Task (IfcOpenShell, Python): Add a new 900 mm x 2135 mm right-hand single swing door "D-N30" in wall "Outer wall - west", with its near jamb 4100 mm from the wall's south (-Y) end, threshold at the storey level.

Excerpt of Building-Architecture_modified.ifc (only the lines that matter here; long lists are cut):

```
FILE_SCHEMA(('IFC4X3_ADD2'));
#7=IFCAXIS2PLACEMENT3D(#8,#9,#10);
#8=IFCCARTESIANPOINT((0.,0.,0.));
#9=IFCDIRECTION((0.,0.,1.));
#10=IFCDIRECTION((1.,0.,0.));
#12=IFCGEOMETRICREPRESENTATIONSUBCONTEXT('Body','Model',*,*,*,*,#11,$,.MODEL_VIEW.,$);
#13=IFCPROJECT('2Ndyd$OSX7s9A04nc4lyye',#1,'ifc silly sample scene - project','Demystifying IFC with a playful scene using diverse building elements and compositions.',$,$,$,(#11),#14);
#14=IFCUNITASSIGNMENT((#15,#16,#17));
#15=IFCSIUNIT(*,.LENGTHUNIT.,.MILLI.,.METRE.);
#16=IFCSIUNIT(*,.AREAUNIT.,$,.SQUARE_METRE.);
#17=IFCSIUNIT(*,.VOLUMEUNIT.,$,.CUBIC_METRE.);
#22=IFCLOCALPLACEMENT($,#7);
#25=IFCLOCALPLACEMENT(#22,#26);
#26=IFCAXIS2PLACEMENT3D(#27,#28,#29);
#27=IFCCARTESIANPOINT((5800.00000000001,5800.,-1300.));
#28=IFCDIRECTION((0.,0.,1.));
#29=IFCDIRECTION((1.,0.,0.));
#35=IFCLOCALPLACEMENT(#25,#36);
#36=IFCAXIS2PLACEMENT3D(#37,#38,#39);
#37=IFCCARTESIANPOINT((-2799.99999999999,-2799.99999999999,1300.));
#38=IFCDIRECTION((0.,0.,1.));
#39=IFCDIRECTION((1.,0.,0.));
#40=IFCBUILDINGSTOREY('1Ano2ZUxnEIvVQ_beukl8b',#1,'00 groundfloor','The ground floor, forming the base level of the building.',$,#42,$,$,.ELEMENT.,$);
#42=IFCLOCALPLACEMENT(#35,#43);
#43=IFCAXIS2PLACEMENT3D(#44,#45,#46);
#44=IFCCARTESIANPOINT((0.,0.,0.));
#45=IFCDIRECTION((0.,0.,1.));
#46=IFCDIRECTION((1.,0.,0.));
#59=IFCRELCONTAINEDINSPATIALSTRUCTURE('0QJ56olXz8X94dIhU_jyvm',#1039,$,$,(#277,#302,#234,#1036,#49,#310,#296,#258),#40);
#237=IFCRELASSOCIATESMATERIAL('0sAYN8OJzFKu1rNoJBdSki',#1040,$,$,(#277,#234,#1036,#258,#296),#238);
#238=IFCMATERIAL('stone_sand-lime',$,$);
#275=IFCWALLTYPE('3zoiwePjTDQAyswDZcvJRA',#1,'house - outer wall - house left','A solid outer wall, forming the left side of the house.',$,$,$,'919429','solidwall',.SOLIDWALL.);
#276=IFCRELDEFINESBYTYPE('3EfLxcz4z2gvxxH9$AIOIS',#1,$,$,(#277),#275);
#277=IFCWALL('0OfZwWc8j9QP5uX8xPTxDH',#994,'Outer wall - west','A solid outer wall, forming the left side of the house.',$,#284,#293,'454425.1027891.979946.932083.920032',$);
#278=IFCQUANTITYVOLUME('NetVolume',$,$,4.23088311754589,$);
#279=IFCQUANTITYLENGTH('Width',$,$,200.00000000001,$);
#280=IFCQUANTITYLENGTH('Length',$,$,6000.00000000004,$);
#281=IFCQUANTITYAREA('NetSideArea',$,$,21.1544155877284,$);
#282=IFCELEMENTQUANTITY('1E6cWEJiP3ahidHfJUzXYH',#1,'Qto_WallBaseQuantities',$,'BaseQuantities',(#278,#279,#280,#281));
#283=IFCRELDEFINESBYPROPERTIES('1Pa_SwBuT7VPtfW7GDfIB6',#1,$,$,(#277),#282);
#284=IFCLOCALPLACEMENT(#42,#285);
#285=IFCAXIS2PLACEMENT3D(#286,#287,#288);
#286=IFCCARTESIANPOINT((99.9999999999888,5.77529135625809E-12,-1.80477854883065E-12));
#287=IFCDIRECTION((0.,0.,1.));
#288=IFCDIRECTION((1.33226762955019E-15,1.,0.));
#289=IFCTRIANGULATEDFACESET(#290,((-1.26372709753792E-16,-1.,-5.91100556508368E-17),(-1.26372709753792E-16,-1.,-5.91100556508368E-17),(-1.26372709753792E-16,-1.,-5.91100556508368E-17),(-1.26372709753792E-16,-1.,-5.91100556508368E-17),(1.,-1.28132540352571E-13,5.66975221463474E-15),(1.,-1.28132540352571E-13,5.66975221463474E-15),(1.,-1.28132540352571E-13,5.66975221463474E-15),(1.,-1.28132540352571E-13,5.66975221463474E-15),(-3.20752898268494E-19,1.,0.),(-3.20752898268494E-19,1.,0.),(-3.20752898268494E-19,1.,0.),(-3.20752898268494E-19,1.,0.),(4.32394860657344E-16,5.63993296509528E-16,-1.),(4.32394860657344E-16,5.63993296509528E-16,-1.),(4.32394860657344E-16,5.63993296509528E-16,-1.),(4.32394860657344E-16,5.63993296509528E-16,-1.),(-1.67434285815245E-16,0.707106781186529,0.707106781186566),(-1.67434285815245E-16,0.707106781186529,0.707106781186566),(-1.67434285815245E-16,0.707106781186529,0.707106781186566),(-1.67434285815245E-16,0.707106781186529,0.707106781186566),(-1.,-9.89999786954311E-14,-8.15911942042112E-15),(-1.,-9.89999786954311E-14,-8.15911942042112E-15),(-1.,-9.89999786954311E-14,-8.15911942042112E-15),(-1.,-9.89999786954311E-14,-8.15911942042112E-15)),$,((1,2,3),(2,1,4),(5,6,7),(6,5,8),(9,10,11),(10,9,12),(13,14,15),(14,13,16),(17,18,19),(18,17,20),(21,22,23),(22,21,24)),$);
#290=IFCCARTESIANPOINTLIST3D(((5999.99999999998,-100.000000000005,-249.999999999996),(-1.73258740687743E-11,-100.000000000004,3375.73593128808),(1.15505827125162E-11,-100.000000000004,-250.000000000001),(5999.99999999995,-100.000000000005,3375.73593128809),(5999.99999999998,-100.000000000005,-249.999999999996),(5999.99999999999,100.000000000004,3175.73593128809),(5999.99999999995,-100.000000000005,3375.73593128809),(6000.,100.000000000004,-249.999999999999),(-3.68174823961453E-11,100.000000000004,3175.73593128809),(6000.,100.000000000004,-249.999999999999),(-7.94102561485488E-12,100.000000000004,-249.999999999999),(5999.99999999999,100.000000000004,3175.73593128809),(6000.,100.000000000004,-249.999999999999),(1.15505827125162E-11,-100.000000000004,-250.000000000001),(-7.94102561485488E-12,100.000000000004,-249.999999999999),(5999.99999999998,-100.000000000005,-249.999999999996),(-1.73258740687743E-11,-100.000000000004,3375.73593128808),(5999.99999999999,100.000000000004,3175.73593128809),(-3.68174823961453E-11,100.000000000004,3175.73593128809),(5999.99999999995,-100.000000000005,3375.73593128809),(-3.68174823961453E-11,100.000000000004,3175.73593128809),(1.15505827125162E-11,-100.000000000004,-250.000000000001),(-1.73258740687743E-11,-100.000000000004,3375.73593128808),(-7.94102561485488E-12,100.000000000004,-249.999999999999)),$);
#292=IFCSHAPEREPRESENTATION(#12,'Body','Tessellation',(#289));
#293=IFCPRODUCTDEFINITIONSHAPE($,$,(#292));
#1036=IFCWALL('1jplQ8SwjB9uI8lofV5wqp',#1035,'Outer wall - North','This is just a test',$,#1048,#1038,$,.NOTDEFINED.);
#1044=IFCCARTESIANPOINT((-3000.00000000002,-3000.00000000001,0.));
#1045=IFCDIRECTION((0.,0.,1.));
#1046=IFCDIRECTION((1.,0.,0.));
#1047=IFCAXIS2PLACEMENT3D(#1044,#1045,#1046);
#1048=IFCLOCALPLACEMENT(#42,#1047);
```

```python
import numpy as np
import ifcopenshell
import ifcopenshell.api.feature
import ifcopenshell.api.geometry
import ifcopenshell.api.pset
import ifcopenshell.api.root
import ifcopenshell.api.spatial
import ifcopenshell.geom
import ifcopenshell.util.element
import ifcopenshell.util.placement
import ifcopenshell.util.representation
import ifcopenshell.util.shape
import ifcopenshell.util.unit

model = ifcopenshell.open("Building-Architecture_modified.ifc")
unit_scale = ifcopenshell.util.unit.calculate_unit_scale(model)
area_scale = ifcopenshell.util.unit.calculate_unit_scale(model, "AREAUNIT")
volume_scale = ifcopenshell.util.unit.calculate_unit_scale(model, "VOLUMEUNIT")
settings = ifcopenshell.geom.settings()


def volume(element):
    """Net volume in cubic metres, openings subtracted."""
    shape = ifcopenshell.geom.create_shape(settings, element)
    return ifcopenshell.util.shape.get_volume(shape.geometry)


wall = model.by_guid("0OfZwWc8j9QP5uX8xPTxDH")
storey = ifcopenshell.util.element.get_container(wall, ifc_class="IfcBuildingStorey")
context = ifcopenshell.util.representation.get_context(model, "Model", "Body", "MODEL_VIEW")
before = volume(wall)

width, height, from_end, sill = 0.9, 2.135, 4.1, 0.0  # metres

# The wall runs along its own X axis, and the end named is its -X end.
wall_shape = ifcopenshell.geom.create_shape(settings, wall)
x, y, z = ifcopenshell.util.shape.get_vertices(wall_shape.geometry).T
start = x.min() + from_end
face, thickness = float(y.min()), float(y.max() - y.min())
wall_matrix = ifcopenshell.util.placement.get_local_placement(wall.ObjectPlacement)
level = ifcopenshell.util.placement.get_local_placement(storey.ObjectPlacement)[2, 3]


def in_wall(x, y):
    """Placement at x, y metres in the wall's axes, at sill height."""
    matrix = wall_matrix.copy()
    matrix[:, 3] = wall_matrix @ np.array([x / unit_scale, y / unit_scale, 0.0, 1.0])
    matrix[2, 3] = level + sill / unit_scale
    return matrix


# Opening: a box that overshoots both wall faces by 50 mm.
opening = ifcopenshell.api.root.create_entity(model, ifc_class="IfcOpeningElement", predefined_type="OPENING")
box = ifcopenshell.api.geometry.add_wall_representation(
    model, context=context, length=width, height=height, thickness=thickness + 0.1
)
ifcopenshell.api.geometry.assign_representation(model, product=opening, representation=box)
ifcopenshell.api.geometry.edit_object_placement(model, product=opening, matrix=in_wall(start, face - 0.05), is_si=False)
ifcopenshell.api.feature.add_feature(model, feature=opening, element=wall)

door = ifcopenshell.api.root.create_entity(model, ifc_class="IfcDoor", name="D-N30", predefined_type="DOOR")
door.OverallWidth, door.OverallHeight = width / unit_scale, height / unit_scale
door.OperationType = "SINGLE_SWING_RIGHT"
body = ifcopenshell.api.geometry.add_door_representation(
    model,
    context=context,
    overall_width=door.OverallWidth,
    overall_height=door.OverallHeight,
    operation_type="SINGLE_SWING_RIGHT",
    lining_properties={"LiningDepth": thickness / unit_scale, "ThresholdDepth": thickness / unit_scale},
)
ifcopenshell.api.geometry.assign_representation(model, product=door, representation=body)
ifcopenshell.api.spatial.assign_container(model, products=[door], relating_structure=storey)
ifcopenshell.api.feature.add_filling(model, opening=opening, element=door)

# The lining spans the wall, so the door starts at the wall face.
ifcopenshell.api.geometry.edit_object_placement(model, product=door, matrix=in_wall(start, face), is_si=False)

after = volume(wall)

# Update the wall's stored quantities.
qto = model.by_id(ifcopenshell.util.element.get_pset(wall, "Qto_WallBaseQuantities", should_inherit=False)["id"])
ifcopenshell.api.pset.edit_qto(model, qto=qto, properties={
    "NetVolume": after / volume_scale,
    "NetSideArea": after / thickness / area_scale,
})

print(f"wall volume {before:.3f} -> {after:.3f} m3")

model.write("Building-Architecture_modified_updated.ifc")
```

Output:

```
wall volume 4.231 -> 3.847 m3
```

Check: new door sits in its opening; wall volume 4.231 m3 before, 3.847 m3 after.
